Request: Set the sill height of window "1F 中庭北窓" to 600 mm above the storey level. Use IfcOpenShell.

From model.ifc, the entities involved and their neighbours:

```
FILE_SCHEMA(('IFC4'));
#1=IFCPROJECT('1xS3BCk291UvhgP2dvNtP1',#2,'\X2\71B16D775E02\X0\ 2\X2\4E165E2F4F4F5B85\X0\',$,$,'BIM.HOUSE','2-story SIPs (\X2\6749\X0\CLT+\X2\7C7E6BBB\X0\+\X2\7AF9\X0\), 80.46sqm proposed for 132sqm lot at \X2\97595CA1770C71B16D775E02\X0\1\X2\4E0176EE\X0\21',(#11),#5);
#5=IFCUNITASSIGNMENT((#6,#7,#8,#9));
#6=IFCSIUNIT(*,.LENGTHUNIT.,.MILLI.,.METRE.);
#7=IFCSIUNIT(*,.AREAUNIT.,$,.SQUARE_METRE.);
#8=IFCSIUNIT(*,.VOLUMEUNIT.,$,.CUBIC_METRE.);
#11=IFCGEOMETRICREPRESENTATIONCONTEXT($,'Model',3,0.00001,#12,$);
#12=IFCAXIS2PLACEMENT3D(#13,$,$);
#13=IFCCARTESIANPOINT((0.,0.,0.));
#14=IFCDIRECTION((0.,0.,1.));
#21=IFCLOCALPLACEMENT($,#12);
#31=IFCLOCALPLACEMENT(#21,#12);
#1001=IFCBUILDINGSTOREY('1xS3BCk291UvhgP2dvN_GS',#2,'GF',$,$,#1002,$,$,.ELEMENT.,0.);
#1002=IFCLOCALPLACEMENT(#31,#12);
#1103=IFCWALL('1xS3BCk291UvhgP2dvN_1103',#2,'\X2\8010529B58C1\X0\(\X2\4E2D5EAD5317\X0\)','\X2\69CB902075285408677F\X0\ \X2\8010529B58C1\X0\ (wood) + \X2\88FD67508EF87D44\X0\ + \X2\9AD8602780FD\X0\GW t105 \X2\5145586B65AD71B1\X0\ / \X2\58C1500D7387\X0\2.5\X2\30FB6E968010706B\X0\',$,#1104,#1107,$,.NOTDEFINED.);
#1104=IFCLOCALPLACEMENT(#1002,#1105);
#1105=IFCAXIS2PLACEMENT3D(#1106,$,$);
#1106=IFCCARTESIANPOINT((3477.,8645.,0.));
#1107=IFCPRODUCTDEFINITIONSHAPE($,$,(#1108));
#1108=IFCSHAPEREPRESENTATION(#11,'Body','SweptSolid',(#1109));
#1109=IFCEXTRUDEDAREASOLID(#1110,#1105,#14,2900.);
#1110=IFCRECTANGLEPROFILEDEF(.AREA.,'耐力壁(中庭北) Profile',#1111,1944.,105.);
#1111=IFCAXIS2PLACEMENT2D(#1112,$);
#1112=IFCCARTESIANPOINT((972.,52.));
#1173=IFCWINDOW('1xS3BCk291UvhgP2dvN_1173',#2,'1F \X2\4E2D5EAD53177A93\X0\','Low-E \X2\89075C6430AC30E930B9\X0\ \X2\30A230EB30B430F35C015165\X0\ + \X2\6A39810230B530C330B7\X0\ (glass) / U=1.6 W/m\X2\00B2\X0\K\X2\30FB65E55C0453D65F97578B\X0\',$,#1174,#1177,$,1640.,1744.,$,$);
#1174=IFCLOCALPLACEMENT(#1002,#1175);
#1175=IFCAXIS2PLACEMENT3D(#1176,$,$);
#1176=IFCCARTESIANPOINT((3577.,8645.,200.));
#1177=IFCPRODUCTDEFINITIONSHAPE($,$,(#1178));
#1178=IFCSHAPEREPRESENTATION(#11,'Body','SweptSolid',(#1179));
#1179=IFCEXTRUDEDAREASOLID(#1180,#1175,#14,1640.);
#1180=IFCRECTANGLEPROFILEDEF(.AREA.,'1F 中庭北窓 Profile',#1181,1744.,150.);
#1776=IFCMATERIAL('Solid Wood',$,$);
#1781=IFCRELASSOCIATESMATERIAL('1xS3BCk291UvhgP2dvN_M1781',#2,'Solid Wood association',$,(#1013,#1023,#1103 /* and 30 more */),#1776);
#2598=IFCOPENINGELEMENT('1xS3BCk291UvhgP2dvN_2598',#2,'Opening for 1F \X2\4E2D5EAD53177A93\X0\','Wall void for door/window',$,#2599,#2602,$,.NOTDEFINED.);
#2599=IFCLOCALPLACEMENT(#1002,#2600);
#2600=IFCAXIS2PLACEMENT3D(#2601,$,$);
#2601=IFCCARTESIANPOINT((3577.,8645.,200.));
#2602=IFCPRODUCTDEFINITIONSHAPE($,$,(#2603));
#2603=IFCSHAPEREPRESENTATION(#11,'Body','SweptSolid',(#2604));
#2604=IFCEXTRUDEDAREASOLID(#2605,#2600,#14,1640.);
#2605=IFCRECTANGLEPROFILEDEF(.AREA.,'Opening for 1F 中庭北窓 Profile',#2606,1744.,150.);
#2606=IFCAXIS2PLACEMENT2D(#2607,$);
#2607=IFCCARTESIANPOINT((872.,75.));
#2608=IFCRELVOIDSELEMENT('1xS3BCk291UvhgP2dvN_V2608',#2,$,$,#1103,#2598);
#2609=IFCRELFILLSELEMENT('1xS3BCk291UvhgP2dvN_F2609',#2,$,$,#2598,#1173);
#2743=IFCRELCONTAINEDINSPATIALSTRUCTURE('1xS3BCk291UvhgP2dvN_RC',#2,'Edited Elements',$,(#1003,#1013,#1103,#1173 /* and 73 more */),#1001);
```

```python
import numpy as np
import ifcopenshell
import ifcopenshell.api.geometry
import ifcopenshell.geom
import ifcopenshell.util.element
import ifcopenshell.util.placement
import ifcopenshell.util.shape
import ifcopenshell.util.unit

model = ifcopenshell.open("model.ifc")
unit_scale = ifcopenshell.util.unit.calculate_unit_scale(model)

window = model.by_guid("1xS3BCk291UvhgP2dvN_1173")
opening = window.FillsVoids[0].RelatingOpeningElement
storey = ifcopenshell.util.element.get_container(window, ifc_class="IfcBuildingStorey")
level = ifcopenshell.util.placement.get_local_placement(storey.ObjectPlacement)[2, 3]

# The opening's origin need not be at the sill, so measure its lowest point.
shape = ifcopenshell.geom.create_shape(ifcopenshell.geom.settings(), opening)
bottom = ifcopenshell.util.shape.get_shape_bottom_elevation(shape, shape.geometry) / unit_scale
dz = level + 0.6 / unit_scale - bottom

shift = np.array([0.0, 0.0, dz])
# The window is not placed relative to its opening, so move both.
for product in (opening, window):
    matrix = ifcopenshell.util.placement.get_local_placement(product.ObjectPlacement)
    matrix[:3, 3] += shift
    ifcopenshell.api.geometry.edit_object_placement(model, product=product, matrix=matrix, is_si=False)

print(f"moved by {dz * unit_scale:+.3f} m")

model.write("model_edited.ifc")
```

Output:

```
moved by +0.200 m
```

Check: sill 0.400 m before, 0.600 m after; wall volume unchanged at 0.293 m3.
